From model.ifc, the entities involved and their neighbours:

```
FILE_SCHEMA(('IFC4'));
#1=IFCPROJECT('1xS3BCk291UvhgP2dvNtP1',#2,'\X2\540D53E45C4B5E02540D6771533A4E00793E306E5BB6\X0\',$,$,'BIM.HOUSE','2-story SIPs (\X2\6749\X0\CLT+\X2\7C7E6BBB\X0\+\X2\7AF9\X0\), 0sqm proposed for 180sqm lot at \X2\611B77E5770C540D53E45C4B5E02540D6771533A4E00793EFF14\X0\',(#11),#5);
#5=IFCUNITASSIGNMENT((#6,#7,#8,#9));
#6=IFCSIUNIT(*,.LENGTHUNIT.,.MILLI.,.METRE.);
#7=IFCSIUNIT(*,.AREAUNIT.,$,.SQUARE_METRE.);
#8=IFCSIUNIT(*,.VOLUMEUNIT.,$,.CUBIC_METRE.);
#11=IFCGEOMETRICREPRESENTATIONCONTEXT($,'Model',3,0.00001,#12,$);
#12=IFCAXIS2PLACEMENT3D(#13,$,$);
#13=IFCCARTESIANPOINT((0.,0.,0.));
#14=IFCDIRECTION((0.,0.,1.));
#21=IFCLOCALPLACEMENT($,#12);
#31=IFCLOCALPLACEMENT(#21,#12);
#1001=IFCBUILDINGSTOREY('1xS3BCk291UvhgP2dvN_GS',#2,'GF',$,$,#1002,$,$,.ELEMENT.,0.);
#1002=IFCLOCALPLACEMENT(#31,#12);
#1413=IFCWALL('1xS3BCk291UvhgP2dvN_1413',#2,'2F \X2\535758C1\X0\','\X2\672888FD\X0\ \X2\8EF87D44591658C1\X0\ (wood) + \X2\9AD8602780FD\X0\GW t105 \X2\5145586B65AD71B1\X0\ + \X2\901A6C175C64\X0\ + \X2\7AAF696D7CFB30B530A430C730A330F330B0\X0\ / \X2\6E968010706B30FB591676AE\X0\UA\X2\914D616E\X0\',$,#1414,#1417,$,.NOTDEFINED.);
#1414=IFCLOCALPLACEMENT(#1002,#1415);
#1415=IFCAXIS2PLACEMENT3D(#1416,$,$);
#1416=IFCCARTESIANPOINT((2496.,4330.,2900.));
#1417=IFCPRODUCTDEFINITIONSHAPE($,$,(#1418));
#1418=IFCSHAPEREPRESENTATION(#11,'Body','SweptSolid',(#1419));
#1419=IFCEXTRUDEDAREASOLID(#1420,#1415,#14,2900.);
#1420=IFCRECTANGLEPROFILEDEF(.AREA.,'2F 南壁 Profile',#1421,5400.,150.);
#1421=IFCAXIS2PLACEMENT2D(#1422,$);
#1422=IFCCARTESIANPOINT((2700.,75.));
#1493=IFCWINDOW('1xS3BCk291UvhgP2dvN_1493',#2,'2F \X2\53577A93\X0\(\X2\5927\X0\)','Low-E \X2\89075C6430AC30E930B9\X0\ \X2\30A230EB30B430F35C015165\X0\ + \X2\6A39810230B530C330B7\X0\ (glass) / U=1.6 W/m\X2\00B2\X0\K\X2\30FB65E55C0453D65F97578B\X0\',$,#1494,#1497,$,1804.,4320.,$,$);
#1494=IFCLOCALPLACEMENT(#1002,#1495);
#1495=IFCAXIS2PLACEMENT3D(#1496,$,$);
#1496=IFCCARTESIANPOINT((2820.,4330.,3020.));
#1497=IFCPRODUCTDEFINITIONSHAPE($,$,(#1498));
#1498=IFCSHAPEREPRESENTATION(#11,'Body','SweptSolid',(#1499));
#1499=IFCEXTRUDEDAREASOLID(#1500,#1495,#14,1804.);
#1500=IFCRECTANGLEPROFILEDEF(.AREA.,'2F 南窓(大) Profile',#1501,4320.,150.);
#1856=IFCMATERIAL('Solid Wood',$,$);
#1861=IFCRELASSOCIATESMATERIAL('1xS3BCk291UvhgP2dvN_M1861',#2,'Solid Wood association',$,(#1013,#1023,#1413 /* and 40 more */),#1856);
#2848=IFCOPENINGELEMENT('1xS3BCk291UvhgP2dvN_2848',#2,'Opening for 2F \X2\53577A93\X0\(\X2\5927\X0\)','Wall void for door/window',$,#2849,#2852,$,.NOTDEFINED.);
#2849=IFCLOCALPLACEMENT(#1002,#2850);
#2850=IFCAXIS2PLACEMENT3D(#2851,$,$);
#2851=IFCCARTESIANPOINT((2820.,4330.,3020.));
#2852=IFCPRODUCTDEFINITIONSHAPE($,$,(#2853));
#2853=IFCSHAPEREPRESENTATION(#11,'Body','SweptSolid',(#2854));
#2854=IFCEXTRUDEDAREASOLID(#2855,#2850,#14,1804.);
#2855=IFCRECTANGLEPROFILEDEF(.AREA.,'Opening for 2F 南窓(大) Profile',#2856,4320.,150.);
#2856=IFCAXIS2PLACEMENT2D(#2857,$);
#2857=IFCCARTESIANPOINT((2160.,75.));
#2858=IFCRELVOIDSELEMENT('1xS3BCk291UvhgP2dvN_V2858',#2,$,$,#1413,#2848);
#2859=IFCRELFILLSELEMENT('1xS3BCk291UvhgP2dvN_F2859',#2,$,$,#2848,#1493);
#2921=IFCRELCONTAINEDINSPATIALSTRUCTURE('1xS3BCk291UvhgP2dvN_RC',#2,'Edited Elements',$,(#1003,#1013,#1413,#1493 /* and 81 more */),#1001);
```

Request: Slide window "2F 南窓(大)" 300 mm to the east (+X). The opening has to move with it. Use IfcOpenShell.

```python
import ifcopenshell
import ifcopenshell.api.geometry
import ifcopenshell.util.placement

model = ifcopenshell.open("model.ifc")

window = model.by_guid("1xS3BCk291UvhgP2dvN_1493")
opening = window.FillsVoids[0].RelatingOpeningElement
wall = opening.VoidsElements[0].RelatingBuildingElement

wall_matrix = ifcopenshell.util.placement.get_local_placement(wall.ObjectPlacement)
shift = wall_matrix[:3, 0] * 300.0
before = ifcopenshell.util.placement.get_local_placement(window.ObjectPlacement)[:3, 3].copy()

# The window is not placed relative to its opening, so move both.
for product in (opening, window):
    matrix = ifcopenshell.util.placement.get_local_placement(product.ObjectPlacement)
    matrix[:3, 3] += shift
    ifcopenshell.api.geometry.edit_object_placement(model, product=product, matrix=matrix, is_si=False)

after = ifcopenshell.util.placement.get_local_placement(window.ObjectPlacement)[:3, 3]
print("window moved by", (after - before).round(3) + 0.0)

model.write("model-out.ifc")
```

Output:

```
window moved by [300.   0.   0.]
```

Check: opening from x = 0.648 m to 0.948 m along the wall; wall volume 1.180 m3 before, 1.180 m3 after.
